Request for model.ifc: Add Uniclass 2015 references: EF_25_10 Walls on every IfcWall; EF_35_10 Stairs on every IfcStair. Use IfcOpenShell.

First a look at what the model holds.

```python
import ifcopenshell

model = ifcopenshell.open("model.ifc")
print(model.schema)
print("classifications:", [c.Name for c in model.by_type("IfcClassification")])
for ifc_class in ("IfcDoor", "IfcRoof", "IfcStair", "IfcWall", "IfcWindow"):
    print(ifc_class, len(model.by_type(ifc_class)))
```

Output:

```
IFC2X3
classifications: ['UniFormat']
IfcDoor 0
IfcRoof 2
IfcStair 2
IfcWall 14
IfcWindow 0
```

```python
import ifcopenshell
import ifcopenshell.api.classification

model = ifcopenshell.open("model.ifc")

# IFC2X3 requires Source and Edition and has no link from the project to the system.
system = model.create_entity("IfcClassification", Source="NBS", Edition="2015", Name="Uniclass 2015")

codes = {
    "IfcWall": ("EF_25_10", "Walls"),
    "IfcStair": ("EF_35_10", "Stairs"),
}
for ifc_class, (code, name) in codes.items():
    products = model.by_type(ifc_class)
    ifcopenshell.api.classification.add_reference(
        model, products=products, classification=system, identification=code, name=name
    )
    print(code, len(products))

model.write("model_rev.ifc")
```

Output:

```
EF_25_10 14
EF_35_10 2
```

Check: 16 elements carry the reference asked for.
